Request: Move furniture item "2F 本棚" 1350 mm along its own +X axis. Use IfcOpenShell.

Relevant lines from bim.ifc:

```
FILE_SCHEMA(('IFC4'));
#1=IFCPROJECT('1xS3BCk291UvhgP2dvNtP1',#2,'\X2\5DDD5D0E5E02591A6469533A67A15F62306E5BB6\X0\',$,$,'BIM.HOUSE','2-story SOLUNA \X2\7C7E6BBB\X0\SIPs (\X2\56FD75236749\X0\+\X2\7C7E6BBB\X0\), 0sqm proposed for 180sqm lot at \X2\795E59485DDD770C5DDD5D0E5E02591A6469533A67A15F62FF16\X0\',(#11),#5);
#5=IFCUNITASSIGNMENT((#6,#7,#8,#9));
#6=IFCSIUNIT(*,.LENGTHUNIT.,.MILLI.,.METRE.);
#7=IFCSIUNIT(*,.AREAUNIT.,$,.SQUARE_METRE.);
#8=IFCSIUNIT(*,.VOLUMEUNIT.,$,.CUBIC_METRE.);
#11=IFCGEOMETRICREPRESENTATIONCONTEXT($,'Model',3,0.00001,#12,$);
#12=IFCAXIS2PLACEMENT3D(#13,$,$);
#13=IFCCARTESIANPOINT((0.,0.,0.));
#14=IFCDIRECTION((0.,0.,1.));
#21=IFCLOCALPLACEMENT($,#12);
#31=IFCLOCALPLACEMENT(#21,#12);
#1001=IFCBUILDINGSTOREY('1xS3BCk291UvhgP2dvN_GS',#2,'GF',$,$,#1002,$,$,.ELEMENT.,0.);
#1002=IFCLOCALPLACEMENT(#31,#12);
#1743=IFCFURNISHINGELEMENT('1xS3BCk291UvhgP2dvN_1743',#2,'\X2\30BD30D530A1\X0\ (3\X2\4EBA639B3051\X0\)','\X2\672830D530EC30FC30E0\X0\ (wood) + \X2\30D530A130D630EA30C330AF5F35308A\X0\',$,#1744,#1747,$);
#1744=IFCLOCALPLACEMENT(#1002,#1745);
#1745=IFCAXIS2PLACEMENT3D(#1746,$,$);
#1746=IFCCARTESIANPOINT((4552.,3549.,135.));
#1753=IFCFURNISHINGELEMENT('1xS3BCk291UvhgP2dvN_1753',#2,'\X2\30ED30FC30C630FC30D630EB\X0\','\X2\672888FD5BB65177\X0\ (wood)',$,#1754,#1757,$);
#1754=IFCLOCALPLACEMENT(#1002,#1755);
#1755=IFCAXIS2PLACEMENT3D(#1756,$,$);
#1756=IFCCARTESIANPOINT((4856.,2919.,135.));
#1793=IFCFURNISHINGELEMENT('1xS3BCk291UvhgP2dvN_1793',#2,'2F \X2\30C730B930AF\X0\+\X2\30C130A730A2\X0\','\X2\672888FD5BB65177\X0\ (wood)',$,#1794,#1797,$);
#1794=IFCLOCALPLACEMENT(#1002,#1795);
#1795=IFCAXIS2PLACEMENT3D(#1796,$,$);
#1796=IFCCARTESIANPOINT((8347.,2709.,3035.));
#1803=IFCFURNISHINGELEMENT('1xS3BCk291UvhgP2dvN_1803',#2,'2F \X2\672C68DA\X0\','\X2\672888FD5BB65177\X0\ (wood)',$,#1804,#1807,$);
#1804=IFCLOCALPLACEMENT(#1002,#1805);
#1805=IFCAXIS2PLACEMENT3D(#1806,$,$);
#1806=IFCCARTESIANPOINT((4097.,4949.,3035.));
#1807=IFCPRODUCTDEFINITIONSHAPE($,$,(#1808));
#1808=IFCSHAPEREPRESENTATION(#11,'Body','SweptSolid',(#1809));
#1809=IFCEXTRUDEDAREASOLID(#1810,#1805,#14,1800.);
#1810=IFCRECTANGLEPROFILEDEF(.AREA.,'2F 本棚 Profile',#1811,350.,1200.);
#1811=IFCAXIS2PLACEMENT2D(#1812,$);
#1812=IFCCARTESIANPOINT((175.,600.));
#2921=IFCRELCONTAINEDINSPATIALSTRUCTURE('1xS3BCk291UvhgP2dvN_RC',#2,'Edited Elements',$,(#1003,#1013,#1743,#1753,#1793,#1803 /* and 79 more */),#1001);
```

```python
import ifcopenshell
import ifcopenshell.api.geometry
import ifcopenshell.util.placement
import ifcopenshell.util.unit

model = ifcopenshell.open("bim.ifc")
unit_scale = ifcopenshell.util.unit.calculate_unit_scale(model)

item = model.by_id(1803)
matrix = ifcopenshell.util.placement.get_local_placement(item.ObjectPlacement)
matrix[:3, 3] += matrix[:3, 0] * 1.35 / unit_scale
ifcopenshell.api.geometry.edit_object_placement(model, product=item, matrix=matrix, is_si=False)

print(ifcopenshell.util.placement.get_local_placement(item.ObjectPlacement).round(3) + 0.0)

model.write("bim_edited.ifc")
```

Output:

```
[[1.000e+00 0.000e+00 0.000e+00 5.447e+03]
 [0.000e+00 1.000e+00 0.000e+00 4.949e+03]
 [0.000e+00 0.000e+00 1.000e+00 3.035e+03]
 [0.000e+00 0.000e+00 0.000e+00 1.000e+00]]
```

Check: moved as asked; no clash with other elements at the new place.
